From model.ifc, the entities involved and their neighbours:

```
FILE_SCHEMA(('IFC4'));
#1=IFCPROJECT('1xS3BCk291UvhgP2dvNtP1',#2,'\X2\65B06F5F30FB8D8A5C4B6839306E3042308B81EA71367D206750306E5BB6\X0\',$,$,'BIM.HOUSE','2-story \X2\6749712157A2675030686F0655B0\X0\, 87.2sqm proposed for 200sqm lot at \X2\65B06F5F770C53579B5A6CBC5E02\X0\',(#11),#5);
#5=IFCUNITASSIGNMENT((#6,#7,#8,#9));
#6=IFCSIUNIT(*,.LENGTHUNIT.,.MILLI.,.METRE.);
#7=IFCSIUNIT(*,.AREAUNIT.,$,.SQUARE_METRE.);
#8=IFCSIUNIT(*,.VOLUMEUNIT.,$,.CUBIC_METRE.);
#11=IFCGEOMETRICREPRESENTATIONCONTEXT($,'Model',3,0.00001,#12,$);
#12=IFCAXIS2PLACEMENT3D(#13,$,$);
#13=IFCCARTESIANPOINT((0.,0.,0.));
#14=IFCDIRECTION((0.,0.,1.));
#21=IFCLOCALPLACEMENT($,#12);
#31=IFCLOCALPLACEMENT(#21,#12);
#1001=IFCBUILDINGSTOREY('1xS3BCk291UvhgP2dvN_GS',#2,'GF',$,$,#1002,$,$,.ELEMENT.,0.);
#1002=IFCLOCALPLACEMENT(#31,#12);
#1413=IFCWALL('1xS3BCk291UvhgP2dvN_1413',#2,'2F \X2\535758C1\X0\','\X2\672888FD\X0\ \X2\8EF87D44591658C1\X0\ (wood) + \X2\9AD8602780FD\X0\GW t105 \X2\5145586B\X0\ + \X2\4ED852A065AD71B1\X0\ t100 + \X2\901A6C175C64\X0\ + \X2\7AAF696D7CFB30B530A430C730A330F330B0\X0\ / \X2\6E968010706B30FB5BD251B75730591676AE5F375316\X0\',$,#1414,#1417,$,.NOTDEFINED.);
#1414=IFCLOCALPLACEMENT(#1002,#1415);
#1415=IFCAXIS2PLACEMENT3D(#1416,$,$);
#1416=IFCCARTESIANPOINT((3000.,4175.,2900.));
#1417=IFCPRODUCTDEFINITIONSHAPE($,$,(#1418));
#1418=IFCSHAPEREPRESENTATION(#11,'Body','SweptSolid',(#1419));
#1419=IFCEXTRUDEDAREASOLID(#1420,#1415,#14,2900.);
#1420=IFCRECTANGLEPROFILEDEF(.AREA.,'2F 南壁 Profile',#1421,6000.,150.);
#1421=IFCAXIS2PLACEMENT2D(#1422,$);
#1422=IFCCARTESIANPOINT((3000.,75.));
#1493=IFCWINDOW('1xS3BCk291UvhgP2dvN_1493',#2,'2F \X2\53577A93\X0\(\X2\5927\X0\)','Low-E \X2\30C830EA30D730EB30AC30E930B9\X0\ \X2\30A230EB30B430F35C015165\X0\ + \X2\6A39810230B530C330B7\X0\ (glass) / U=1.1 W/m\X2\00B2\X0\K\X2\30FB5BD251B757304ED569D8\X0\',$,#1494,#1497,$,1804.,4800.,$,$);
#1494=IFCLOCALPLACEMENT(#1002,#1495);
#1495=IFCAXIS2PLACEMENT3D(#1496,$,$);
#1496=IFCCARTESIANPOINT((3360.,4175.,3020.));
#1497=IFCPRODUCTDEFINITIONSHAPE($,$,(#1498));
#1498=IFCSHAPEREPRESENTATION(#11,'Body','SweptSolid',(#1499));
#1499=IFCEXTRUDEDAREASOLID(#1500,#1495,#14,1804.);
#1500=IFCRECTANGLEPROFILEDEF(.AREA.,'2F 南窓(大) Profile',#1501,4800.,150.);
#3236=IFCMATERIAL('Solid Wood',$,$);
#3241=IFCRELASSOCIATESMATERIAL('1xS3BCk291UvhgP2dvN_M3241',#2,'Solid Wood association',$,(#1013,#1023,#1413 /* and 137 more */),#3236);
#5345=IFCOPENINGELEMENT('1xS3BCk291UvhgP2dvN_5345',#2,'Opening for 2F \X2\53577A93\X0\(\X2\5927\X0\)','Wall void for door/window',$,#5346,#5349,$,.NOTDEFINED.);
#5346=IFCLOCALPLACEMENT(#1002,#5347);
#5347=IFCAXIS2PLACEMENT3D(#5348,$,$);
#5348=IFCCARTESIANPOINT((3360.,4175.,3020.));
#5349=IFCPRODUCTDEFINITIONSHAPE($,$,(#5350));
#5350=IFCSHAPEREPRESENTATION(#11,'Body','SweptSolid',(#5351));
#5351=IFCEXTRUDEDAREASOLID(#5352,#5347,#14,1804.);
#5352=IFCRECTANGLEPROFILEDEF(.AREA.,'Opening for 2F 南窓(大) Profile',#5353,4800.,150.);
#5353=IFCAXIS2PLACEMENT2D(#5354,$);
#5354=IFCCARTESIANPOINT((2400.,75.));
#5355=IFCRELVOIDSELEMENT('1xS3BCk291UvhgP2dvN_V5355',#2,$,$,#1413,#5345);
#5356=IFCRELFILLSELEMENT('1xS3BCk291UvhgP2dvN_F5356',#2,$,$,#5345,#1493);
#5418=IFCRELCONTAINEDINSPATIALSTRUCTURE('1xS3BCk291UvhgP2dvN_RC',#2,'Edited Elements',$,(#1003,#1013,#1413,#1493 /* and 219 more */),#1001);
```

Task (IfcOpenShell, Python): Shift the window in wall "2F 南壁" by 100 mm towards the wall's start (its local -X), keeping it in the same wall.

```python
import ifcopenshell
import ifcopenshell.api.geometry
import ifcopenshell.util.placement

model = ifcopenshell.open("model.ifc")

window = model.by_guid("1xS3BCk291UvhgP2dvN_1493")
opening = window.FillsVoids[0].RelatingOpeningElement
wall = opening.VoidsElements[0].RelatingBuildingElement

wall_matrix = ifcopenshell.util.placement.get_local_placement(wall.ObjectPlacement)
shift = wall_matrix[:3, 0] * -100.0
before = ifcopenshell.util.placement.get_local_placement(window.ObjectPlacement)[:3, 3].copy()

# The window is not placed relative to its opening, so move both.
for product in (opening, window):
    matrix = ifcopenshell.util.placement.get_local_placement(product.ObjectPlacement)
    matrix[:3, 3] += shift
    ifcopenshell.api.geometry.edit_object_placement(model, product=product, matrix=matrix, is_si=False)

after = ifcopenshell.util.placement.get_local_placement(window.ObjectPlacement)[:3, 3]
print("window moved by", (after - before).round(3) + 0.0)

model.write("model_rev.ifc")
```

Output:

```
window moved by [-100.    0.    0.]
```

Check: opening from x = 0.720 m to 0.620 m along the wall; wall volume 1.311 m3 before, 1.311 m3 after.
